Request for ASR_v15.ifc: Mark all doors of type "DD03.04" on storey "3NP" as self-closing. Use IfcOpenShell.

First a look at what the model holds.

```python
import ifcopenshell
import ifcopenshell.util.element

model = ifcopenshell.open("ASR_v15.ifc")
print(model.schema)
storey = next(s for s in model.by_type("IfcBuildingStorey") if s.Name == "3NP")
doors = [e for e in ifcopenshell.util.element.get_decomposition(storey) if e.is_a("IfcDoor")]
seen = {}
for e in doors:
    element_type = ifcopenshell.util.element.get_type(e)
    key = (element_type.Name if element_type != e and element_type else None, ifcopenshell.util.element.get_pset(e, "Pset_DoorCommon", "SelfClosing"))
    seen[key] = seen.get(key, 0) + 1
for (name, value), count in sorted(seen.items(), key=str):
    print(count, "x", name, "|", value)
```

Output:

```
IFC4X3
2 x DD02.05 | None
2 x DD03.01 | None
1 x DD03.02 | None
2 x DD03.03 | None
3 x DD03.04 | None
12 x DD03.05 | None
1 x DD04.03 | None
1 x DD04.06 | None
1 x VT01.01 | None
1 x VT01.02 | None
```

```python
import ifcopenshell
import ifcopenshell.api.pset
import ifcopenshell.util.element

model = ifcopenshell.open("ASR_v15.ifc")

storey = next(s for s in model.by_type("IfcBuildingStorey") if s.Name == "3NP")
doors = [e for e in ifcopenshell.util.element.get_decomposition(storey) if e.is_a("IfcDoor")]

count = 0
for e in doors:
    element_type = ifcopenshell.util.element.get_type(e)
    if element_type in (None, e) or element_type.Name != "DD03.04":
        continue
    # add_pset returns the element's existing set when there is one.
    pset = ifcopenshell.api.pset.add_pset(model, product=e, name="Pset_DoorCommon")
    ifcopenshell.api.pset.edit_pset(model, pset=pset, properties={"SelfClosing": True})
    count += 1

print(count, "doors updated")

model.write("ASR_v15-out.ifc")
```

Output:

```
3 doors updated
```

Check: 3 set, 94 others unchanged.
